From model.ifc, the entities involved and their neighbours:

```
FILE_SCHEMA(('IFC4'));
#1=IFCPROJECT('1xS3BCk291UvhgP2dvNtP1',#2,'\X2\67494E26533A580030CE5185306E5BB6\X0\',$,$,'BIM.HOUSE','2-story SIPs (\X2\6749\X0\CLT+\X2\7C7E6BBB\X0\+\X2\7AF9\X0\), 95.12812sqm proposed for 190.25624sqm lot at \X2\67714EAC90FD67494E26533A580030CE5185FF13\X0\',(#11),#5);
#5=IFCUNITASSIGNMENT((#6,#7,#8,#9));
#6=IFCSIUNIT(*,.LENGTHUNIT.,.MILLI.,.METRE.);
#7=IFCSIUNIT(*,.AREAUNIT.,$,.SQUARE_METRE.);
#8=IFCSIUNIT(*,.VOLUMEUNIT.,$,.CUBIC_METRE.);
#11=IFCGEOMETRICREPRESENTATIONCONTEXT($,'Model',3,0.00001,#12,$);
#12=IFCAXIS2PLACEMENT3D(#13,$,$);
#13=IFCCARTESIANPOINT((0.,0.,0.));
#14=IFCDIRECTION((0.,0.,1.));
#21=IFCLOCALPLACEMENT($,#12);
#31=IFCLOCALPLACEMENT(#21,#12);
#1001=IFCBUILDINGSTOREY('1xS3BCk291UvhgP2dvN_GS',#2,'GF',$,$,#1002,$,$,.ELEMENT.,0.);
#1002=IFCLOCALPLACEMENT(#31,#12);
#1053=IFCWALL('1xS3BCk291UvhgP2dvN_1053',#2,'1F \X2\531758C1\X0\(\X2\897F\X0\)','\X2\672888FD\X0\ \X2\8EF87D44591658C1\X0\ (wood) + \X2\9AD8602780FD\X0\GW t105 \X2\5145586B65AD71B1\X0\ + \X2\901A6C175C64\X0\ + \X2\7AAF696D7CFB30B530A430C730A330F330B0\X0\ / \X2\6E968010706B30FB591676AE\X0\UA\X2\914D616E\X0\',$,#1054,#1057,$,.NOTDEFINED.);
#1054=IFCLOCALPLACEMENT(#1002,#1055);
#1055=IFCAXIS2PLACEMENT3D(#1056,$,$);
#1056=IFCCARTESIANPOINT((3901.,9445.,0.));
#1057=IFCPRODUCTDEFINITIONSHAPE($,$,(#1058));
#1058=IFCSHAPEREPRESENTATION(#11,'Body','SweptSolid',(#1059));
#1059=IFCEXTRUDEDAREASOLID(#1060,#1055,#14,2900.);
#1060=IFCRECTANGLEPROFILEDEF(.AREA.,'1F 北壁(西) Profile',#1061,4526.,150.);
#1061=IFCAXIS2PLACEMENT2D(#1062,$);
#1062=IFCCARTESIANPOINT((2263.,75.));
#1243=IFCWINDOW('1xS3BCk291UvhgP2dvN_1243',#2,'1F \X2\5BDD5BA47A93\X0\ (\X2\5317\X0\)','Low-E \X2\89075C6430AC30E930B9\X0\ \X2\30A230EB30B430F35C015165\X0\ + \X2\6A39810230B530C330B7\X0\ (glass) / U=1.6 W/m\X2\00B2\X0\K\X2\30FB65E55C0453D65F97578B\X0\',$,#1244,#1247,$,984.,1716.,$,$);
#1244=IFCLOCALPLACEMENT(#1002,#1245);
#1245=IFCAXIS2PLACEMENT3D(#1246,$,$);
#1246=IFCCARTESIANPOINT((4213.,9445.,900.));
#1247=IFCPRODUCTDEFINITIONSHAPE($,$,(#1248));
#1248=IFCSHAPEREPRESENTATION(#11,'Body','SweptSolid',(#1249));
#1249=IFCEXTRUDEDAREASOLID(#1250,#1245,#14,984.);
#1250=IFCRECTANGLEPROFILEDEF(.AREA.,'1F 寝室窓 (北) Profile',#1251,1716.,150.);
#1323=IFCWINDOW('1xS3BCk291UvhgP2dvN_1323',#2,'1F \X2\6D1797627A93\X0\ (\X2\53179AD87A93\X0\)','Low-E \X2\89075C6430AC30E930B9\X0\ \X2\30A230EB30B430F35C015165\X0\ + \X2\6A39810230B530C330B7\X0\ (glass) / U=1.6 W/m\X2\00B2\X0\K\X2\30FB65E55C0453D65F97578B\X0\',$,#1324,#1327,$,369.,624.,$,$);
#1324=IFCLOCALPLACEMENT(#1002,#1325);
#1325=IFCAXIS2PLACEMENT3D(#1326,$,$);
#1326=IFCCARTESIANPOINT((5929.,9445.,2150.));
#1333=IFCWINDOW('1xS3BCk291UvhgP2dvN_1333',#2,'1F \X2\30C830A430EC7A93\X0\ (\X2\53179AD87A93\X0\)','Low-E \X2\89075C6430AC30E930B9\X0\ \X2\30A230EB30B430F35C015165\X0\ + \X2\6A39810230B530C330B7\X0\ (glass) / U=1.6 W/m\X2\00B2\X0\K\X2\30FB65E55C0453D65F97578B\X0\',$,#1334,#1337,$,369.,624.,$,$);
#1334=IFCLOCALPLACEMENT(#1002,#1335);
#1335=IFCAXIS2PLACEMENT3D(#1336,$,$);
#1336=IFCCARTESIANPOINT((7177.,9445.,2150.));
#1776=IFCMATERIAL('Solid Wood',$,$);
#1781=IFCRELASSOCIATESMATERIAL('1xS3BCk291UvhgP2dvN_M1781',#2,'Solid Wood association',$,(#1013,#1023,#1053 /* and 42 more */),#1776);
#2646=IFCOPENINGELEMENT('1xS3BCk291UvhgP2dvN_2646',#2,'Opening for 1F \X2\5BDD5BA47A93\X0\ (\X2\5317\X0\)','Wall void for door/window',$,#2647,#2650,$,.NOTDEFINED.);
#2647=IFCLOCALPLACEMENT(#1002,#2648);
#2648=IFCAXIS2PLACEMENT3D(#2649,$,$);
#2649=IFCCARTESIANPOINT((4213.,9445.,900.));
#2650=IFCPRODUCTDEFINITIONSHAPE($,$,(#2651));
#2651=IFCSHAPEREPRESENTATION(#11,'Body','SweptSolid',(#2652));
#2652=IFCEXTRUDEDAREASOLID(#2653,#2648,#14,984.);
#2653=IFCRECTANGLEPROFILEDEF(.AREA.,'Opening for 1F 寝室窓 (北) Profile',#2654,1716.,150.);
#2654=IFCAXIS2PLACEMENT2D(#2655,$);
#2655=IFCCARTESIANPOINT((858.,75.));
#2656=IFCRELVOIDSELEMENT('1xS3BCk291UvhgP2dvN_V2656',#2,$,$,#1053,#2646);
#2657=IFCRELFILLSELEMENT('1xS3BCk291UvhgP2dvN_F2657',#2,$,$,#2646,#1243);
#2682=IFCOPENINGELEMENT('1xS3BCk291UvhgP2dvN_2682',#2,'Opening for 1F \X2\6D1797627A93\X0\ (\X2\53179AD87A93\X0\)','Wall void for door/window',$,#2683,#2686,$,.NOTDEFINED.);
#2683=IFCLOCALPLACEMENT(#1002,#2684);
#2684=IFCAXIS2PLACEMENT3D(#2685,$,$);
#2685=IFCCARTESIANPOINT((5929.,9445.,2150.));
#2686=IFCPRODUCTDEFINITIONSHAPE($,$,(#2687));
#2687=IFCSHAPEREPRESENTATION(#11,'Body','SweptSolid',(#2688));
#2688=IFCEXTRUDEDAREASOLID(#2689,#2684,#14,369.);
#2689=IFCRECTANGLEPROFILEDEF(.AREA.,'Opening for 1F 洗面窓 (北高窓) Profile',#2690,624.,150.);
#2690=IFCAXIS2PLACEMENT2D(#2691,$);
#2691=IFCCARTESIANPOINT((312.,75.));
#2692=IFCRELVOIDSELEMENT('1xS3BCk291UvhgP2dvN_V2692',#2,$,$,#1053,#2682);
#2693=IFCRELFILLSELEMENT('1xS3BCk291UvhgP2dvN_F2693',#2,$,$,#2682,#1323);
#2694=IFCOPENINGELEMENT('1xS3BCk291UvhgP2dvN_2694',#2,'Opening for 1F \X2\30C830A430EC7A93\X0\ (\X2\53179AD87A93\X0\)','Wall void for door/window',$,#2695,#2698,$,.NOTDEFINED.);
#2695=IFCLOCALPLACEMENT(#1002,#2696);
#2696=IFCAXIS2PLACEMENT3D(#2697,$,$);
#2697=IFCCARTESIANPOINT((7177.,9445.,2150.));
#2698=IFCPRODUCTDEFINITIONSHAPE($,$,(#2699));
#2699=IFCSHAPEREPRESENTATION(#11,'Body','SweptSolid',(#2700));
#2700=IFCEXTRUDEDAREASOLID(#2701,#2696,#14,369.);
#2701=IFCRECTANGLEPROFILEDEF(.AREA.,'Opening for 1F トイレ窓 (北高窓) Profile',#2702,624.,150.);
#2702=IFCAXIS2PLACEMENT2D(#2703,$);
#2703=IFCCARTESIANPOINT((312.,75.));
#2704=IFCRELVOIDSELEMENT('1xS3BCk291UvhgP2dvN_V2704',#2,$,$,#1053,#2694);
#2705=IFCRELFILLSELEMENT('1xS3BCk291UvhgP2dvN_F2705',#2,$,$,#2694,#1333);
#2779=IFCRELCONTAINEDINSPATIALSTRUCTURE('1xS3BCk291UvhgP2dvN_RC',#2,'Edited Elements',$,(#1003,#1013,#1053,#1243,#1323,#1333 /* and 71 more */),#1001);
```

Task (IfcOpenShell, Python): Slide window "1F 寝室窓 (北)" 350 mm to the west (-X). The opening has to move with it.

```python
import ifcopenshell
import ifcopenshell.api.geometry
import ifcopenshell.util.placement
import ifcopenshell.util.unit

model = ifcopenshell.open("model.ifc")
unit_scale = ifcopenshell.util.unit.calculate_unit_scale(model)

window = model.by_guid("1xS3BCk291UvhgP2dvN_1243")
opening = window.FillsVoids[0].RelatingOpeningElement
wall = opening.VoidsElements[0].RelatingBuildingElement

wall_matrix = ifcopenshell.util.placement.get_local_placement(wall.ObjectPlacement)
shift = wall_matrix[:3, 0] * -0.35 / unit_scale
before = ifcopenshell.util.placement.get_local_placement(window.ObjectPlacement)[:3, 3].copy()

# The window is not placed relative to its opening, so move both.
for product in (opening, window):
    matrix = ifcopenshell.util.placement.get_local_placement(product.ObjectPlacement)
    matrix[:3, 3] += shift
    ifcopenshell.api.geometry.edit_object_placement(model, product=product, matrix=matrix, is_si=False)

after = ifcopenshell.util.placement.get_local_placement(window.ObjectPlacement)[:3, 3]
print("window moved by", (after - before).round(3) + 0.0)

model.write("model_v2.ifc")
```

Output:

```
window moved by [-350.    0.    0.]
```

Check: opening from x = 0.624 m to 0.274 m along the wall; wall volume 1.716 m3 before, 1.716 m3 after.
